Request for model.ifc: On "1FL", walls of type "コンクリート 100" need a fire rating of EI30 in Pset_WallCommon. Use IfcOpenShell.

First a look at what the model holds.

```python
import ifcopenshell
import ifcopenshell.util.element

model = ifcopenshell.open("model.ifc")
print(model.schema)
storey = next(s for s in model.by_type("IfcBuildingStorey") if s.Name == "1FL")
walls = [e for e in ifcopenshell.util.element.get_decomposition(storey) if e.is_a("IfcWall")]
seen = {}
for e in walls:
    element_type = ifcopenshell.util.element.get_type(e)
    key = (element_type.Name if element_type != e and element_type else None, ifcopenshell.util.element.get_pset(e, "Pset_WallCommon", "FireRating"))
    seen[key] = seen.get(key, 0) + 1
for (name, value), count in sorted(seen.items(), key=str):
    print(count, "x", name, "|", value)
```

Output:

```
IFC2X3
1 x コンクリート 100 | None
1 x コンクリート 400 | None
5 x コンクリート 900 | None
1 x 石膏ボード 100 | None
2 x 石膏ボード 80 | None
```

```python
import ifcopenshell
import ifcopenshell.api.pset
import ifcopenshell.util.element

model = ifcopenshell.open("model.ifc")

storey = next(s for s in model.by_type("IfcBuildingStorey") if s.Name == "1FL")
walls = [e for e in ifcopenshell.util.element.get_decomposition(storey) if e.is_a("IfcWall")]

count = 0
for e in walls:
    element_type = ifcopenshell.util.element.get_type(e)
    if element_type in (None, e) or element_type.Name != "コンクリート 100":
        continue
    # add_pset returns the element's existing set when there is one.
    pset = ifcopenshell.api.pset.add_pset(model, product=e, name="Pset_WallCommon")
    ifcopenshell.api.pset.edit_pset(model, pset=pset, properties={"FireRating": "EI30"})
    count += 1

print(count, "walls updated")

model.write("model_rev.ifc")
```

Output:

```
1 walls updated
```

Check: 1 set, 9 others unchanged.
